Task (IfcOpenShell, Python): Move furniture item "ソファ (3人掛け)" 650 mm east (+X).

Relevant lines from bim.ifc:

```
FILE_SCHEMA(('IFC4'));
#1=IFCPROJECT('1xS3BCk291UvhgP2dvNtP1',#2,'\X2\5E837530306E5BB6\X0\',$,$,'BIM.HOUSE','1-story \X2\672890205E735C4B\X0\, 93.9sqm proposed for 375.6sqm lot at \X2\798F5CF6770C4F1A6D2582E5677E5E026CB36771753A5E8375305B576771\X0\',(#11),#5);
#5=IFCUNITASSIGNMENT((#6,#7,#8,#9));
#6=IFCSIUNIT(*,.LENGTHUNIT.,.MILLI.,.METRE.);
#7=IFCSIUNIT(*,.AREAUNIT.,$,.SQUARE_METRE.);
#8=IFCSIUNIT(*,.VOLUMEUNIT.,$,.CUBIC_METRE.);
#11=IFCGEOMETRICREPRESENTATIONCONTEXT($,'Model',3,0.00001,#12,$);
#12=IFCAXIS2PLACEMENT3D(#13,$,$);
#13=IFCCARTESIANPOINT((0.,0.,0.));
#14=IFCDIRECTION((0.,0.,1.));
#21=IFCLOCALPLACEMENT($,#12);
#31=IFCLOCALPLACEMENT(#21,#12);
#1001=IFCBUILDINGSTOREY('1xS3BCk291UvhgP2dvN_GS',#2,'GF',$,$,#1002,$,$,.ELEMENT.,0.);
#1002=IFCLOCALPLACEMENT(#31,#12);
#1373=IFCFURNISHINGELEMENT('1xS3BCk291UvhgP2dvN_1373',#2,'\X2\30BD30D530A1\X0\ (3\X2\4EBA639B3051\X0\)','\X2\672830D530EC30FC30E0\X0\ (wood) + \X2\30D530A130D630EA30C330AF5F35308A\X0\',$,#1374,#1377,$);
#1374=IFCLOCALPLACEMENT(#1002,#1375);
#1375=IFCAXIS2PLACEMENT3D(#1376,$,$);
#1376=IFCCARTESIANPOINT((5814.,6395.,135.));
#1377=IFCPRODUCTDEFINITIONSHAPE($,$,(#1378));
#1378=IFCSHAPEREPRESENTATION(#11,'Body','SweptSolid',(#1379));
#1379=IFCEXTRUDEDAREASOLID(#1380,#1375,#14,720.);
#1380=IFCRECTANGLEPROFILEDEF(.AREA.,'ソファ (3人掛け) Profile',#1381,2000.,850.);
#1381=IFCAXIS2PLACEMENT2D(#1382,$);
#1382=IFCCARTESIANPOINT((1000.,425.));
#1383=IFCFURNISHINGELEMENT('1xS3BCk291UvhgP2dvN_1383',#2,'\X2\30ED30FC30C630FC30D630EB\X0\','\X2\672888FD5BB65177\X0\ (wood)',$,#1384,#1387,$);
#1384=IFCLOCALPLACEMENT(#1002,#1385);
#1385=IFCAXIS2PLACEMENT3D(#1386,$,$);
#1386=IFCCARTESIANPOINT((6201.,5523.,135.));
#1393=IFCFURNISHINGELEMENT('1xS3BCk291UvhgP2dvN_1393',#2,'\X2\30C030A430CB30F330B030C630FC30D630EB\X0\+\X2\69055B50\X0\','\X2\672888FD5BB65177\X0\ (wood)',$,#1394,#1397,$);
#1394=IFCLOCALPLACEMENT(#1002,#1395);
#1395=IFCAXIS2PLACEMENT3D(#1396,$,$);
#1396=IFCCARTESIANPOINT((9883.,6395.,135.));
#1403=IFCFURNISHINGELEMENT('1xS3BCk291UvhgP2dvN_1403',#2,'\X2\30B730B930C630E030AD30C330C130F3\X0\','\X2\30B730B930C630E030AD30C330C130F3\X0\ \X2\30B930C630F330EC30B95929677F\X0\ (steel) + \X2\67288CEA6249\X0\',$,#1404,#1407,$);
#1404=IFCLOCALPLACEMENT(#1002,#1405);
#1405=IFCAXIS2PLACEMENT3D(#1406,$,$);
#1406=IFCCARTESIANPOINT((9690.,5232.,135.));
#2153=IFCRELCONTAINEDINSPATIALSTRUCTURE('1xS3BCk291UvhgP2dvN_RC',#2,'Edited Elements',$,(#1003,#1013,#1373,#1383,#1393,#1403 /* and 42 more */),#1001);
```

```python
import ifcopenshell
import ifcopenshell.api.geometry
import ifcopenshell.util.placement
import ifcopenshell.util.unit

model = ifcopenshell.open("bim.ifc")
unit_scale = ifcopenshell.util.unit.calculate_unit_scale(model)

item = model.by_guid("1xS3BCk291UvhgP2dvN_1373")
matrix = ifcopenshell.util.placement.get_local_placement(item.ObjectPlacement)
matrix[0, 3] += 0.65 / unit_scale
ifcopenshell.api.geometry.edit_object_placement(model, product=item, matrix=matrix, is_si=False)

print(ifcopenshell.util.placement.get_local_placement(item.ObjectPlacement).round(3) + 0.0)

model.write("bim-out.ifc")
```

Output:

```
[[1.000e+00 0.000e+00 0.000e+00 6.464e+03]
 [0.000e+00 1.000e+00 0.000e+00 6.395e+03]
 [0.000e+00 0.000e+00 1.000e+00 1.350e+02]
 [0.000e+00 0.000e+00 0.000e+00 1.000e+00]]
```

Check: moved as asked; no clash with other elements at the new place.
